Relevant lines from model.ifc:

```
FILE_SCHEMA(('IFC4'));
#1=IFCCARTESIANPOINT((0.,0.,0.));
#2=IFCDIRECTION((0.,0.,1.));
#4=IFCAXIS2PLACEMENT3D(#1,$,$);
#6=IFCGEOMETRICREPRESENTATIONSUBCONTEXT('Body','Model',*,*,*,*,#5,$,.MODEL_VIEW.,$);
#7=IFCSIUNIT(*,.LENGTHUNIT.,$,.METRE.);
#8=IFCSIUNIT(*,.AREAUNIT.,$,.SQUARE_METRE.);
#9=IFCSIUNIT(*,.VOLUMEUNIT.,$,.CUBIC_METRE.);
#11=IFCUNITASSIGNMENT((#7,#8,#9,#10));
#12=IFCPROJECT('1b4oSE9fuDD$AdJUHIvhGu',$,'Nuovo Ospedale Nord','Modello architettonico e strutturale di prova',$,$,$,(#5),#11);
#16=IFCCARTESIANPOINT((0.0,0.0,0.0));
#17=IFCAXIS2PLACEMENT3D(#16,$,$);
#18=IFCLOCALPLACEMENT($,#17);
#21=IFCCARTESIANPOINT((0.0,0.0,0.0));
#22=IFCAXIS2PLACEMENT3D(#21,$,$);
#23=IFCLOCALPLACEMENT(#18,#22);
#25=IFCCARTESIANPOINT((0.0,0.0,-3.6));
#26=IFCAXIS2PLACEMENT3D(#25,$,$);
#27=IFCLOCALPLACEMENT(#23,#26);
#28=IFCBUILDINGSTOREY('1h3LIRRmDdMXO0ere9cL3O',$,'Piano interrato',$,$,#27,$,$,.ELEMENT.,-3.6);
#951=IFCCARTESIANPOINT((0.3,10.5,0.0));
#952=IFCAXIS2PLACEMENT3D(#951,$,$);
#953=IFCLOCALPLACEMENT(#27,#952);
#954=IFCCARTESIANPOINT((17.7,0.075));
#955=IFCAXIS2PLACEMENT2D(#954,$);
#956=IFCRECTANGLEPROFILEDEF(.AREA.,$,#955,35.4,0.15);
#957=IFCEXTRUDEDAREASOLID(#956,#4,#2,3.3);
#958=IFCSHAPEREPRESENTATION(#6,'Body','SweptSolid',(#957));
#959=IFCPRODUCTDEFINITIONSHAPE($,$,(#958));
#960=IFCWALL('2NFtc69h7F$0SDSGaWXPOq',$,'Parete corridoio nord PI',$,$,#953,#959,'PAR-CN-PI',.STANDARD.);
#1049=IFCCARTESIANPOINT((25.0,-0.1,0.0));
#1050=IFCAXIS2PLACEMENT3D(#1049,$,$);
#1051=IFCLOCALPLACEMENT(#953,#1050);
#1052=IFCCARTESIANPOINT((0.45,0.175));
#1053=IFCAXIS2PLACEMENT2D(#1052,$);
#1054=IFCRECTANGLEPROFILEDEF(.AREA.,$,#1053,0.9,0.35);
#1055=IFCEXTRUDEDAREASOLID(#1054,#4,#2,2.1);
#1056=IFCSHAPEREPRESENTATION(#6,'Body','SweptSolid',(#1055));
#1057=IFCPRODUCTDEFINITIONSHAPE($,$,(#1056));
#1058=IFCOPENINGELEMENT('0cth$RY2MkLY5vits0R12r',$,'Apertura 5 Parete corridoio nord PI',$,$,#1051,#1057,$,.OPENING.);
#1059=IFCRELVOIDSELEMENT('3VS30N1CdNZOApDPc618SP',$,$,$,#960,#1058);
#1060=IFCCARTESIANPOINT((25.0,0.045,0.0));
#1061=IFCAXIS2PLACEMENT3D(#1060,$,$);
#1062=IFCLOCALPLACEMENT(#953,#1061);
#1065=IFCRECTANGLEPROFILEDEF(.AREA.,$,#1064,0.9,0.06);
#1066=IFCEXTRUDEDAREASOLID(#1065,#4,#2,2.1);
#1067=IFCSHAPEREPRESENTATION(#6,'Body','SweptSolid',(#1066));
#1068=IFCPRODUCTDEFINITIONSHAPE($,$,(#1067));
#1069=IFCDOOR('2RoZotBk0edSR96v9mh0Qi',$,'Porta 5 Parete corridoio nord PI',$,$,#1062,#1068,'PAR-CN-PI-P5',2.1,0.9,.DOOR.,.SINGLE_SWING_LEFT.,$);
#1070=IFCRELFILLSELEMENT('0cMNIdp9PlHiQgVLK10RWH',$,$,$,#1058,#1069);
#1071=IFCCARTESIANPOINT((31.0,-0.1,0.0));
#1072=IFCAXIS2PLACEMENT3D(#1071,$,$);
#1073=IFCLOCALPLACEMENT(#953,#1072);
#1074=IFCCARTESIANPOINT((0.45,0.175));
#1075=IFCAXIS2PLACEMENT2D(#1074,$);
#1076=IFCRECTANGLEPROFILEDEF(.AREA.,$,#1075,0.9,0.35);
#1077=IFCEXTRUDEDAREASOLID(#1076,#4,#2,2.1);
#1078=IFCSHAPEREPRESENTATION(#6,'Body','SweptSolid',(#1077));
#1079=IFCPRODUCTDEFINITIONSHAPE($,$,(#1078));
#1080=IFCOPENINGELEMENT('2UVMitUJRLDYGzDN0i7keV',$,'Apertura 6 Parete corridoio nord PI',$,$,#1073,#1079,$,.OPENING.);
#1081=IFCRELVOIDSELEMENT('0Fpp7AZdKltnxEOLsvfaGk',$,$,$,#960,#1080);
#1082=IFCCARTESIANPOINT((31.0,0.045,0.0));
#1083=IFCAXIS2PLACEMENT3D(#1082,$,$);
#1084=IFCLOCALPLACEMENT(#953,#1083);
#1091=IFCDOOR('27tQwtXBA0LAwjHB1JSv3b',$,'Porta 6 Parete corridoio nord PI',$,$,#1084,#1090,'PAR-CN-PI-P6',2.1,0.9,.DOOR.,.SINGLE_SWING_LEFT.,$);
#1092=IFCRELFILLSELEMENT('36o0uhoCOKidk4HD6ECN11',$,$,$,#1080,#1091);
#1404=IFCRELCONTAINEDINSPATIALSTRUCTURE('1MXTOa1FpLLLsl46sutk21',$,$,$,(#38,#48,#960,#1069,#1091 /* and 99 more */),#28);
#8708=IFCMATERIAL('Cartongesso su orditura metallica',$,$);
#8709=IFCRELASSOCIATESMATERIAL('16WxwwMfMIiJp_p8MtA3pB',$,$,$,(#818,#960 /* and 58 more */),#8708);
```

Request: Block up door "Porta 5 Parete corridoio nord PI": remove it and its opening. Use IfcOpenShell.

```python
import ifcopenshell
import ifcopenshell.api.feature
import ifcopenshell.api.root
import ifcopenshell.geom
import ifcopenshell.util.shape

model = ifcopenshell.open("model.ifc")
settings = ifcopenshell.geom.settings()


def volume(element):
    """Net volume in cubic metres, openings subtracted."""
    shape = ifcopenshell.geom.create_shape(settings, element)
    return ifcopenshell.util.shape.get_volume(shape.geometry)


door = model.by_guid("2RoZotBk0edSR96v9mh0Qi")
opening = door.FillsVoids[0].RelatingOpeningElement
wall = opening.VoidsElements[0].RelatingBuildingElement
before = volume(wall)

ifcopenshell.api.root.remove_product(model, product=door)
ifcopenshell.api.feature.remove_feature(model, feature=opening)

after = volume(wall)

print(f"wall volume {before:.3f} -> {after:.3f} m3")

model.write("model_updated.ifc")
```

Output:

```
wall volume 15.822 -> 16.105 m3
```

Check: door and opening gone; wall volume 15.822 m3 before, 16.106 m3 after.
